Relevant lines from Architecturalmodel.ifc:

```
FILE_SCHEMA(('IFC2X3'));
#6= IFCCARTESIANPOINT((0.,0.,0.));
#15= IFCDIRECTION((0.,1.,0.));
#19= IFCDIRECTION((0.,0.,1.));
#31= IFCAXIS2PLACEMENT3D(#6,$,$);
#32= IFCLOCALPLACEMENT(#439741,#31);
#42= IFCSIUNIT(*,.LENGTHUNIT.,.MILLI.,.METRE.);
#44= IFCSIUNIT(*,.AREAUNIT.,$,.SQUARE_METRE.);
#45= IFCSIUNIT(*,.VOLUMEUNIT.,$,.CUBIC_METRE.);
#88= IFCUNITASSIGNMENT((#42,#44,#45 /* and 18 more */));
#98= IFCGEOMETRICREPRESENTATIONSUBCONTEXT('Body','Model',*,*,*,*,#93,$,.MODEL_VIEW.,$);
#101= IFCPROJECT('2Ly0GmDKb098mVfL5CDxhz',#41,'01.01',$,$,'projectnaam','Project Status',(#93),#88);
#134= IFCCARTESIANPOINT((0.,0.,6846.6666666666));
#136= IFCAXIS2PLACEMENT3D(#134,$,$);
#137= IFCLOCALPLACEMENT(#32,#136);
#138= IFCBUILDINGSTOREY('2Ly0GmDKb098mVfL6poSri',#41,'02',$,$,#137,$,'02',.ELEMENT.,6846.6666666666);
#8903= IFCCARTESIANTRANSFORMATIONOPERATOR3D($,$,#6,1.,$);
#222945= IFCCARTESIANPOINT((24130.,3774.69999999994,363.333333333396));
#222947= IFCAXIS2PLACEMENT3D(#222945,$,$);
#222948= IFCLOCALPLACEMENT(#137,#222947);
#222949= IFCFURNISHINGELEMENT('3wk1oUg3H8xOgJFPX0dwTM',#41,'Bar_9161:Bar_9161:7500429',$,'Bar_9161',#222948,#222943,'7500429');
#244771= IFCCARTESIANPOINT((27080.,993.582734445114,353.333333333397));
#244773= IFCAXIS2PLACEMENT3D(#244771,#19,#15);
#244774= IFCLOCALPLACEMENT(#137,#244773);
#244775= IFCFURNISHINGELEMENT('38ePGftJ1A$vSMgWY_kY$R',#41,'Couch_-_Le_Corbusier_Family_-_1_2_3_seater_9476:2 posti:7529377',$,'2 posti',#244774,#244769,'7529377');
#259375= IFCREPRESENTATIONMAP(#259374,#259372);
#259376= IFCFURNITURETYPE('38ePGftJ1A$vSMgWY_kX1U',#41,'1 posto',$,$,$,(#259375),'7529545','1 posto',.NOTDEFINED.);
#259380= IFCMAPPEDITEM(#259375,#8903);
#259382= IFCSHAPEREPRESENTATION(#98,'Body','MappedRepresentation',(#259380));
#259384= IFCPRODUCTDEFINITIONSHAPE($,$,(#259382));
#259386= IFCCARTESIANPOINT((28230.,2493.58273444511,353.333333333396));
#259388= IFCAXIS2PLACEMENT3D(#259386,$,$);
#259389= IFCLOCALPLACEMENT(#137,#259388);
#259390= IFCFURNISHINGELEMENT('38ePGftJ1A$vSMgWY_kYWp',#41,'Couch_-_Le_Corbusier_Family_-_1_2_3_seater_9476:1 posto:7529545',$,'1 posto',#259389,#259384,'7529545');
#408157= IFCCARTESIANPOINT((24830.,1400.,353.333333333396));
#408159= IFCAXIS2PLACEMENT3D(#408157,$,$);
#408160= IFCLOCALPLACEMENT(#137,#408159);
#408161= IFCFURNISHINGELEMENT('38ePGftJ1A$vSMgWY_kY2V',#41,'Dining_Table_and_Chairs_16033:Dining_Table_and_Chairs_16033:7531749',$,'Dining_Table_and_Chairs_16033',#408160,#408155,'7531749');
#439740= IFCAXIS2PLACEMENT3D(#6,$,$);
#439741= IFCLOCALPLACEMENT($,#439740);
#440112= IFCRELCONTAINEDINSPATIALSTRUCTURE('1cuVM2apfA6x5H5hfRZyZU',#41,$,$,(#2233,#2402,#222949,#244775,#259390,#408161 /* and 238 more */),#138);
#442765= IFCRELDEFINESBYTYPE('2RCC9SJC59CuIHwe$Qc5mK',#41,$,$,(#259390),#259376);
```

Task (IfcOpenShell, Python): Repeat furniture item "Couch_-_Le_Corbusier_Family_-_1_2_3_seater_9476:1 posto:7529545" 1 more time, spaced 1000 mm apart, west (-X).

```python
import numpy as np
import ifcopenshell
import ifcopenshell.api.geometry
import ifcopenshell.api.root
import ifcopenshell.util.element
import ifcopenshell.util.placement
import ifcopenshell.util.unit

model = ifcopenshell.open("Architecturalmodel.ifc")
unit_scale = ifcopenshell.util.unit.calculate_unit_scale(model)

source = model.by_guid("38ePGftJ1A$vSMgWY_kYWp")
base = ifcopenshell.util.placement.get_local_placement(source.ObjectPlacement)
step = np.array([-1.0, 0.0, 0.0]) * 1 / unit_scale

for i in range(1, 2):
    copy = ifcopenshell.api.root.copy_class(model, product=source)
    copy.Representation = ifcopenshell.util.element.copy_deep(
        model, source.Representation, exclude=["IfcGeometricRepresentationContext", "IfcRepresentationMap"]
    )
    copy.Name = "Couch_-_Le_Corbusier_Family_-_1_2_3_seater_9476:1 posto"
    copy.Tag = None
    matrix = base.copy()
    matrix[:3, 3] += i * step
    print("added at", matrix[:3, 3].round(3) + 0.0)
    ifcopenshell.api.geometry.edit_object_placement(model, product=copy, matrix=matrix, is_si=False)

model.write("Architecturalmodel_v2.ifc")
```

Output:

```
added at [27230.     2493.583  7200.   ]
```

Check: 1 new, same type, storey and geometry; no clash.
